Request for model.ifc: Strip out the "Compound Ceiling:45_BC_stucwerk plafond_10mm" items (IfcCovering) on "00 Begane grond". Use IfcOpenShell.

First a look at what the model holds.

```python
import ifcopenshell
import ifcopenshell.util.element

model = ifcopenshell.open("model.ifc")
print(model.schema)
storey = next(s for s in model.by_type("IfcBuildingStorey") if s.Name == "00 Begane grond")
coverings = [e for e in ifcopenshell.util.element.get_decomposition(storey) if e.is_a("IfcCovering")]
seen = {}
for e in coverings:
    element_type = ifcopenshell.util.element.get_type(e)
    name = element_type.Name if element_type not in (None, e) else None
    seen[name] = seen.get(name, 0) + 1
for name, count in sorted(seen.items(), key=str):
    print(count, "x", name)
```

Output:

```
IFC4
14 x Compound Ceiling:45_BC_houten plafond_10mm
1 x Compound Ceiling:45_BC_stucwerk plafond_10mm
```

```python
import ifcopenshell
import ifcopenshell.api.root
import ifcopenshell.util.element

model = ifcopenshell.open("model.ifc")

storey = next(s for s in model.by_type("IfcBuildingStorey") if s.Name == "00 Begane grond")
coverings = [e for e in ifcopenshell.util.element.get_decomposition(storey) if e.is_a("IfcCovering")]
targets = [e for e in coverings if (t := ifcopenshell.util.element.get_type(e)) not in (None, e) and t.Name == "Compound Ceiling:45_BC_stucwerk plafond_10mm"]

for e in targets:
    ifcopenshell.api.root.remove_product(model, product=e)
print(len(targets), "removed")

model.write("model_edited.ifc")
```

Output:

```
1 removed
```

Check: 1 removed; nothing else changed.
